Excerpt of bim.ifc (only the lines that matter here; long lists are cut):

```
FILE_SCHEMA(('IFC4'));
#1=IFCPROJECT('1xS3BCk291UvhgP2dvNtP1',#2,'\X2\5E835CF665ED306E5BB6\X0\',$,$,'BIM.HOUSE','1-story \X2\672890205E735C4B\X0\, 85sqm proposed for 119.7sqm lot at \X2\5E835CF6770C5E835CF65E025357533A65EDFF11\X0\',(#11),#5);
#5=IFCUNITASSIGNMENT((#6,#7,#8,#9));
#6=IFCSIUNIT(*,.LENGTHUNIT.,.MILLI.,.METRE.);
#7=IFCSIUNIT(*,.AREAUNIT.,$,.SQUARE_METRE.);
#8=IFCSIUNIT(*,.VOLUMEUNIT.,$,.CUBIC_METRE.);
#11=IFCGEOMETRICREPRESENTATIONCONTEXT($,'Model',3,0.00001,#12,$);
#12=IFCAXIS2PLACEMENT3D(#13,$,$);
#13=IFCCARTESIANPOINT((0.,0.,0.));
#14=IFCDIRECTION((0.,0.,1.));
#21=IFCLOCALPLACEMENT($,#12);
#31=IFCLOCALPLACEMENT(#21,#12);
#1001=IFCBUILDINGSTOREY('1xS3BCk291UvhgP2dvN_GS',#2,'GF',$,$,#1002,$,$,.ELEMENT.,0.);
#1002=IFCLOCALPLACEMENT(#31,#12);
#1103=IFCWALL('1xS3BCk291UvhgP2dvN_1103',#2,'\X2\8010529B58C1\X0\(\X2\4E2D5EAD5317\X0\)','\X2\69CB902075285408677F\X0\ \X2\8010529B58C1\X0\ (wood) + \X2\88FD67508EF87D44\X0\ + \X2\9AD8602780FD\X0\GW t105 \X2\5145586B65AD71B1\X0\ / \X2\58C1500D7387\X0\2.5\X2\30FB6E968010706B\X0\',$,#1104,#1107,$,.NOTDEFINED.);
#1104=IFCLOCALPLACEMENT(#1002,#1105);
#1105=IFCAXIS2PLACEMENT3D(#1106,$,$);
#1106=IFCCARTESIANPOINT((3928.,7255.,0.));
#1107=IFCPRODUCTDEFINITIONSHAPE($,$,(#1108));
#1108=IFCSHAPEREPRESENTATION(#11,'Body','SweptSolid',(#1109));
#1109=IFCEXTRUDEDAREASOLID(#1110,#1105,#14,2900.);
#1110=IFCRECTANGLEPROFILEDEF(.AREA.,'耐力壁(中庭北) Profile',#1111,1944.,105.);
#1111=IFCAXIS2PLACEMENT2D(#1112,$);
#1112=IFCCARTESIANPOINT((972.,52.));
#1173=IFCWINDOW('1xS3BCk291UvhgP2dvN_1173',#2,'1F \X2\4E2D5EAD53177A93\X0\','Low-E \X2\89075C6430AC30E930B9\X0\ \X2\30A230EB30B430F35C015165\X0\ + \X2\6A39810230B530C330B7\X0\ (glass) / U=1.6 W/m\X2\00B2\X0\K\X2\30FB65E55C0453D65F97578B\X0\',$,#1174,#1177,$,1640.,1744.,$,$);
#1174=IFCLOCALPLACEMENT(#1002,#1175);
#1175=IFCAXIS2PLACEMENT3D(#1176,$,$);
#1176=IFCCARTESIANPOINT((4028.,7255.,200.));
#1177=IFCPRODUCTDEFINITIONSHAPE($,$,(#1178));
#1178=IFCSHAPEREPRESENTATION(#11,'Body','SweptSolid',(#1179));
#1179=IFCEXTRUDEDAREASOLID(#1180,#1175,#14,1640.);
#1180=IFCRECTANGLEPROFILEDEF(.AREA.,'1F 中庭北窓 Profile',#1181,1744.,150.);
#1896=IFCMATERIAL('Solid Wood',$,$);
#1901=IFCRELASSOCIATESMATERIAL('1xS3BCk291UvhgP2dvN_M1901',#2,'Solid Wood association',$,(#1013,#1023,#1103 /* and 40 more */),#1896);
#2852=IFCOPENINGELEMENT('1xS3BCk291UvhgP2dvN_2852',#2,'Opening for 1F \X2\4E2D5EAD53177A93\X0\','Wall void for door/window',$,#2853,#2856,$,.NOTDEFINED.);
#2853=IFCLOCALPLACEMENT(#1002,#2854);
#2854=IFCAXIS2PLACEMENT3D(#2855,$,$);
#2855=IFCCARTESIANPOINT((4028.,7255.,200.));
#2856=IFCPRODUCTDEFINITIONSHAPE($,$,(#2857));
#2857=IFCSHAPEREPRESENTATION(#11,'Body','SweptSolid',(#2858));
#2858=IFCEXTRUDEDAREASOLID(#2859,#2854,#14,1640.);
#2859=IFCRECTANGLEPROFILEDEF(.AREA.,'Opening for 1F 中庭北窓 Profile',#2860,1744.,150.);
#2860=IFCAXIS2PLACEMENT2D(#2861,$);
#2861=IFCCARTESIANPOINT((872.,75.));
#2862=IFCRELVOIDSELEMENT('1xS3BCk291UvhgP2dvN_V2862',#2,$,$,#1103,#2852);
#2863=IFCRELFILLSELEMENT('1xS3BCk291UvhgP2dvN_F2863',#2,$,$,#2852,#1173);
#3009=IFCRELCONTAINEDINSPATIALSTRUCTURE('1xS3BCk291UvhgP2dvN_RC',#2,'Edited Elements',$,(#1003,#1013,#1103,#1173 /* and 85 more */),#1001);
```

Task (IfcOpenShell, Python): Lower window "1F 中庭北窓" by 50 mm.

```python
import numpy as np
import ifcopenshell
import ifcopenshell.api.geometry
import ifcopenshell.util.placement
import ifcopenshell.util.unit

model = ifcopenshell.open("bim.ifc")
unit_scale = ifcopenshell.util.unit.calculate_unit_scale(model)

window = model.by_guid("1xS3BCk291UvhgP2dvN_1173")
opening = window.FillsVoids[0].RelatingOpeningElement
dz = -50.0

shift = np.array([0.0, 0.0, dz])
# The window is not placed relative to its opening, so move both.
for product in (opening, window):
    matrix = ifcopenshell.util.placement.get_local_placement(product.ObjectPlacement)
    matrix[:3, 3] += shift
    ifcopenshell.api.geometry.edit_object_placement(model, product=product, matrix=matrix, is_si=False)

print(f"moved by {dz * unit_scale:+.3f} m")

model.write("bim-out.ifc")
```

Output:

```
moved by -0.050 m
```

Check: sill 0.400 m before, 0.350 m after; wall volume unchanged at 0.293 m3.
